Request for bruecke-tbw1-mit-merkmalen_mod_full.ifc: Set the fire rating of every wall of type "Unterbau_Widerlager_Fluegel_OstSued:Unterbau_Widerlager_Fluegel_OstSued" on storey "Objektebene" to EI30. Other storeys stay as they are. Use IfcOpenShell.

First a look at what the model holds.

```python
import ifcopenshell
import ifcopenshell.util.element

model = ifcopenshell.open("bruecke-tbw1-mit-merkmalen_mod_full.ifc")
print(model.schema)
storey = next(s for s in model.by_type("IfcBuildingStorey") if s.Name == "Objektebene")
walls = [e for e in ifcopenshell.util.element.get_decomposition(storey) if e.is_a("IfcWall")]
seen = {}
for e in walls:
    element_type = ifcopenshell.util.element.get_type(e)
    key = (element_type.Name if element_type != e and element_type else None, ifcopenshell.util.element.get_pset(e, "Pset_WallCommon", "FireRating"))
    seen[key] = seen.get(key, 0) + 1
for (name, value), count in sorted(seen.items(), key=str):
    print(count, "x", name, "|", value)
```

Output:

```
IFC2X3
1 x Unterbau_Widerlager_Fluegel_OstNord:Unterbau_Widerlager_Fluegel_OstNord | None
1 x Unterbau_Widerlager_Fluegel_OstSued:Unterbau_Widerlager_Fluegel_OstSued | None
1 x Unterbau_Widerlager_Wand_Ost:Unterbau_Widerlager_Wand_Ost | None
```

```python
import ifcopenshell
import ifcopenshell.api.pset
import ifcopenshell.util.element

model = ifcopenshell.open("bruecke-tbw1-mit-merkmalen_mod_full.ifc")

storey = next(s for s in model.by_type("IfcBuildingStorey") if s.Name == "Objektebene")
walls = [e for e in ifcopenshell.util.element.get_decomposition(storey) if e.is_a("IfcWall")]

count = 0
for e in walls:
    element_type = ifcopenshell.util.element.get_type(e)
    if element_type in (None, e) or element_type.Name != "Unterbau_Widerlager_Fluegel_OstSued:Unterbau_Widerlager_Fluegel_OstSued":
        continue
    # add_pset returns the element's existing set when there is one.
    pset = ifcopenshell.api.pset.add_pset(model, product=e, name="Pset_WallCommon")
    ifcopenshell.api.pset.edit_pset(model, pset=pset, properties={"FireRating": "EI30"})
    count += 1

print(count, "walls updated")

model.write("bruecke-tbw1-mit-merkmalen_mod_full_edited.ifc")
```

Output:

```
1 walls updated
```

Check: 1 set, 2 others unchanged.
